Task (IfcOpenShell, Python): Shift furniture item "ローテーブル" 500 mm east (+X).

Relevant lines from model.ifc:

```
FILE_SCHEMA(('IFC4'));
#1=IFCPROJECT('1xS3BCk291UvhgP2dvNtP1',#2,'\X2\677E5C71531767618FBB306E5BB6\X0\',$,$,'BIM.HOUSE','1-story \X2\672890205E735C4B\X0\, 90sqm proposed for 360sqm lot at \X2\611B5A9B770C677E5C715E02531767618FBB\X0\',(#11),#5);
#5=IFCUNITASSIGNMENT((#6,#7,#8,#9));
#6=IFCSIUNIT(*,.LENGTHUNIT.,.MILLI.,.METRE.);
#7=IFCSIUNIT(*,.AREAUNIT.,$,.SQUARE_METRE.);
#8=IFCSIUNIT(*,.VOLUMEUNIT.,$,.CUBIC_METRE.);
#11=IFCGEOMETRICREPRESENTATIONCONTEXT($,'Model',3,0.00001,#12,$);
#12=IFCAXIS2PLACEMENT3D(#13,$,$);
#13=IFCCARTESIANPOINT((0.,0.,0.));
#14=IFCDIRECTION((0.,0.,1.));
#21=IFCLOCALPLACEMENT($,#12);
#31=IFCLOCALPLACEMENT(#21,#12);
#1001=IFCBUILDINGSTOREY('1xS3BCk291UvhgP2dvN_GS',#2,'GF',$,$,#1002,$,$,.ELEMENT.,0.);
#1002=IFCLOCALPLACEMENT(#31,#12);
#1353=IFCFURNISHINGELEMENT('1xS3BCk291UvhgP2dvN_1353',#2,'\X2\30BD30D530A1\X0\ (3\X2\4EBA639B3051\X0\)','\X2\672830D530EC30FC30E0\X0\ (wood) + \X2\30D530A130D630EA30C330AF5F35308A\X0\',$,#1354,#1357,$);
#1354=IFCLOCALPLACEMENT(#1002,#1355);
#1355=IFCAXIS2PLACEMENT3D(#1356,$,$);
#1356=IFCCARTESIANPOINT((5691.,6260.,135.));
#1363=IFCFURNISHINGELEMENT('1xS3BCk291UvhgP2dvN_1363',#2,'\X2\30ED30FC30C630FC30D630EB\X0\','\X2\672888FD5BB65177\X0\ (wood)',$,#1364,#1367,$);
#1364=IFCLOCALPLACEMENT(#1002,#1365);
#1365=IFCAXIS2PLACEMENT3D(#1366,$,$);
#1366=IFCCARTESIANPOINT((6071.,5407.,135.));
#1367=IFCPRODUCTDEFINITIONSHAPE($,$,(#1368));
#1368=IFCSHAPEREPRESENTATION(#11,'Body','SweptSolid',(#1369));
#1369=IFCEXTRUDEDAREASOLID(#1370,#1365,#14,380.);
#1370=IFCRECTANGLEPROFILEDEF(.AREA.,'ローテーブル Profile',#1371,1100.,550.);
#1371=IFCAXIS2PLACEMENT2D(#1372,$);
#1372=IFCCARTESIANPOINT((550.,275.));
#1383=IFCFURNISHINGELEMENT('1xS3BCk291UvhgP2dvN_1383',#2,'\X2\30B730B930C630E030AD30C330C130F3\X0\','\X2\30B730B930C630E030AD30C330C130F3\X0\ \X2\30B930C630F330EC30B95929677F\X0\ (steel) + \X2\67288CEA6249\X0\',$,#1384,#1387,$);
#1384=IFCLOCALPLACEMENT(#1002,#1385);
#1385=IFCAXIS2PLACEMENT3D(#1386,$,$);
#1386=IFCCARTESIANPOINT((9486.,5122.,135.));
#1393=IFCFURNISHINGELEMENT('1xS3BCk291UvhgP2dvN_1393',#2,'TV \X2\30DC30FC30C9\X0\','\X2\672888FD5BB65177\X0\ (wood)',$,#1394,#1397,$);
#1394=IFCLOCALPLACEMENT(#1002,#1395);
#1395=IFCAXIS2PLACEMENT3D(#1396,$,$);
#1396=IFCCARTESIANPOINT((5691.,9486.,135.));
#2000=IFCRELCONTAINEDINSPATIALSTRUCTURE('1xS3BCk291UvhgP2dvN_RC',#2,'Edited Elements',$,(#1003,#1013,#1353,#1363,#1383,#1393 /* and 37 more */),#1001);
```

```python
import ifcopenshell
import ifcopenshell.api.geometry
import ifcopenshell.util.placement

model = ifcopenshell.open("model.ifc")

item = model.by_guid("1xS3BCk291UvhgP2dvN_1363")
matrix = ifcopenshell.util.placement.get_local_placement(item.ObjectPlacement)
matrix[0, 3] += 500.0
ifcopenshell.api.geometry.edit_object_placement(model, product=item, matrix=matrix, is_si=False)

print(ifcopenshell.util.placement.get_local_placement(item.ObjectPlacement).round(3) + 0.0)

model.write("model_rev.ifc")
```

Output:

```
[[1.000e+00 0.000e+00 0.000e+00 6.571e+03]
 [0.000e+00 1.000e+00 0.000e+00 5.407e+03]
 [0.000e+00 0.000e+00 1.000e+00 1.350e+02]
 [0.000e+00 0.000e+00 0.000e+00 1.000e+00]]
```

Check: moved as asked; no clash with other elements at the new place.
